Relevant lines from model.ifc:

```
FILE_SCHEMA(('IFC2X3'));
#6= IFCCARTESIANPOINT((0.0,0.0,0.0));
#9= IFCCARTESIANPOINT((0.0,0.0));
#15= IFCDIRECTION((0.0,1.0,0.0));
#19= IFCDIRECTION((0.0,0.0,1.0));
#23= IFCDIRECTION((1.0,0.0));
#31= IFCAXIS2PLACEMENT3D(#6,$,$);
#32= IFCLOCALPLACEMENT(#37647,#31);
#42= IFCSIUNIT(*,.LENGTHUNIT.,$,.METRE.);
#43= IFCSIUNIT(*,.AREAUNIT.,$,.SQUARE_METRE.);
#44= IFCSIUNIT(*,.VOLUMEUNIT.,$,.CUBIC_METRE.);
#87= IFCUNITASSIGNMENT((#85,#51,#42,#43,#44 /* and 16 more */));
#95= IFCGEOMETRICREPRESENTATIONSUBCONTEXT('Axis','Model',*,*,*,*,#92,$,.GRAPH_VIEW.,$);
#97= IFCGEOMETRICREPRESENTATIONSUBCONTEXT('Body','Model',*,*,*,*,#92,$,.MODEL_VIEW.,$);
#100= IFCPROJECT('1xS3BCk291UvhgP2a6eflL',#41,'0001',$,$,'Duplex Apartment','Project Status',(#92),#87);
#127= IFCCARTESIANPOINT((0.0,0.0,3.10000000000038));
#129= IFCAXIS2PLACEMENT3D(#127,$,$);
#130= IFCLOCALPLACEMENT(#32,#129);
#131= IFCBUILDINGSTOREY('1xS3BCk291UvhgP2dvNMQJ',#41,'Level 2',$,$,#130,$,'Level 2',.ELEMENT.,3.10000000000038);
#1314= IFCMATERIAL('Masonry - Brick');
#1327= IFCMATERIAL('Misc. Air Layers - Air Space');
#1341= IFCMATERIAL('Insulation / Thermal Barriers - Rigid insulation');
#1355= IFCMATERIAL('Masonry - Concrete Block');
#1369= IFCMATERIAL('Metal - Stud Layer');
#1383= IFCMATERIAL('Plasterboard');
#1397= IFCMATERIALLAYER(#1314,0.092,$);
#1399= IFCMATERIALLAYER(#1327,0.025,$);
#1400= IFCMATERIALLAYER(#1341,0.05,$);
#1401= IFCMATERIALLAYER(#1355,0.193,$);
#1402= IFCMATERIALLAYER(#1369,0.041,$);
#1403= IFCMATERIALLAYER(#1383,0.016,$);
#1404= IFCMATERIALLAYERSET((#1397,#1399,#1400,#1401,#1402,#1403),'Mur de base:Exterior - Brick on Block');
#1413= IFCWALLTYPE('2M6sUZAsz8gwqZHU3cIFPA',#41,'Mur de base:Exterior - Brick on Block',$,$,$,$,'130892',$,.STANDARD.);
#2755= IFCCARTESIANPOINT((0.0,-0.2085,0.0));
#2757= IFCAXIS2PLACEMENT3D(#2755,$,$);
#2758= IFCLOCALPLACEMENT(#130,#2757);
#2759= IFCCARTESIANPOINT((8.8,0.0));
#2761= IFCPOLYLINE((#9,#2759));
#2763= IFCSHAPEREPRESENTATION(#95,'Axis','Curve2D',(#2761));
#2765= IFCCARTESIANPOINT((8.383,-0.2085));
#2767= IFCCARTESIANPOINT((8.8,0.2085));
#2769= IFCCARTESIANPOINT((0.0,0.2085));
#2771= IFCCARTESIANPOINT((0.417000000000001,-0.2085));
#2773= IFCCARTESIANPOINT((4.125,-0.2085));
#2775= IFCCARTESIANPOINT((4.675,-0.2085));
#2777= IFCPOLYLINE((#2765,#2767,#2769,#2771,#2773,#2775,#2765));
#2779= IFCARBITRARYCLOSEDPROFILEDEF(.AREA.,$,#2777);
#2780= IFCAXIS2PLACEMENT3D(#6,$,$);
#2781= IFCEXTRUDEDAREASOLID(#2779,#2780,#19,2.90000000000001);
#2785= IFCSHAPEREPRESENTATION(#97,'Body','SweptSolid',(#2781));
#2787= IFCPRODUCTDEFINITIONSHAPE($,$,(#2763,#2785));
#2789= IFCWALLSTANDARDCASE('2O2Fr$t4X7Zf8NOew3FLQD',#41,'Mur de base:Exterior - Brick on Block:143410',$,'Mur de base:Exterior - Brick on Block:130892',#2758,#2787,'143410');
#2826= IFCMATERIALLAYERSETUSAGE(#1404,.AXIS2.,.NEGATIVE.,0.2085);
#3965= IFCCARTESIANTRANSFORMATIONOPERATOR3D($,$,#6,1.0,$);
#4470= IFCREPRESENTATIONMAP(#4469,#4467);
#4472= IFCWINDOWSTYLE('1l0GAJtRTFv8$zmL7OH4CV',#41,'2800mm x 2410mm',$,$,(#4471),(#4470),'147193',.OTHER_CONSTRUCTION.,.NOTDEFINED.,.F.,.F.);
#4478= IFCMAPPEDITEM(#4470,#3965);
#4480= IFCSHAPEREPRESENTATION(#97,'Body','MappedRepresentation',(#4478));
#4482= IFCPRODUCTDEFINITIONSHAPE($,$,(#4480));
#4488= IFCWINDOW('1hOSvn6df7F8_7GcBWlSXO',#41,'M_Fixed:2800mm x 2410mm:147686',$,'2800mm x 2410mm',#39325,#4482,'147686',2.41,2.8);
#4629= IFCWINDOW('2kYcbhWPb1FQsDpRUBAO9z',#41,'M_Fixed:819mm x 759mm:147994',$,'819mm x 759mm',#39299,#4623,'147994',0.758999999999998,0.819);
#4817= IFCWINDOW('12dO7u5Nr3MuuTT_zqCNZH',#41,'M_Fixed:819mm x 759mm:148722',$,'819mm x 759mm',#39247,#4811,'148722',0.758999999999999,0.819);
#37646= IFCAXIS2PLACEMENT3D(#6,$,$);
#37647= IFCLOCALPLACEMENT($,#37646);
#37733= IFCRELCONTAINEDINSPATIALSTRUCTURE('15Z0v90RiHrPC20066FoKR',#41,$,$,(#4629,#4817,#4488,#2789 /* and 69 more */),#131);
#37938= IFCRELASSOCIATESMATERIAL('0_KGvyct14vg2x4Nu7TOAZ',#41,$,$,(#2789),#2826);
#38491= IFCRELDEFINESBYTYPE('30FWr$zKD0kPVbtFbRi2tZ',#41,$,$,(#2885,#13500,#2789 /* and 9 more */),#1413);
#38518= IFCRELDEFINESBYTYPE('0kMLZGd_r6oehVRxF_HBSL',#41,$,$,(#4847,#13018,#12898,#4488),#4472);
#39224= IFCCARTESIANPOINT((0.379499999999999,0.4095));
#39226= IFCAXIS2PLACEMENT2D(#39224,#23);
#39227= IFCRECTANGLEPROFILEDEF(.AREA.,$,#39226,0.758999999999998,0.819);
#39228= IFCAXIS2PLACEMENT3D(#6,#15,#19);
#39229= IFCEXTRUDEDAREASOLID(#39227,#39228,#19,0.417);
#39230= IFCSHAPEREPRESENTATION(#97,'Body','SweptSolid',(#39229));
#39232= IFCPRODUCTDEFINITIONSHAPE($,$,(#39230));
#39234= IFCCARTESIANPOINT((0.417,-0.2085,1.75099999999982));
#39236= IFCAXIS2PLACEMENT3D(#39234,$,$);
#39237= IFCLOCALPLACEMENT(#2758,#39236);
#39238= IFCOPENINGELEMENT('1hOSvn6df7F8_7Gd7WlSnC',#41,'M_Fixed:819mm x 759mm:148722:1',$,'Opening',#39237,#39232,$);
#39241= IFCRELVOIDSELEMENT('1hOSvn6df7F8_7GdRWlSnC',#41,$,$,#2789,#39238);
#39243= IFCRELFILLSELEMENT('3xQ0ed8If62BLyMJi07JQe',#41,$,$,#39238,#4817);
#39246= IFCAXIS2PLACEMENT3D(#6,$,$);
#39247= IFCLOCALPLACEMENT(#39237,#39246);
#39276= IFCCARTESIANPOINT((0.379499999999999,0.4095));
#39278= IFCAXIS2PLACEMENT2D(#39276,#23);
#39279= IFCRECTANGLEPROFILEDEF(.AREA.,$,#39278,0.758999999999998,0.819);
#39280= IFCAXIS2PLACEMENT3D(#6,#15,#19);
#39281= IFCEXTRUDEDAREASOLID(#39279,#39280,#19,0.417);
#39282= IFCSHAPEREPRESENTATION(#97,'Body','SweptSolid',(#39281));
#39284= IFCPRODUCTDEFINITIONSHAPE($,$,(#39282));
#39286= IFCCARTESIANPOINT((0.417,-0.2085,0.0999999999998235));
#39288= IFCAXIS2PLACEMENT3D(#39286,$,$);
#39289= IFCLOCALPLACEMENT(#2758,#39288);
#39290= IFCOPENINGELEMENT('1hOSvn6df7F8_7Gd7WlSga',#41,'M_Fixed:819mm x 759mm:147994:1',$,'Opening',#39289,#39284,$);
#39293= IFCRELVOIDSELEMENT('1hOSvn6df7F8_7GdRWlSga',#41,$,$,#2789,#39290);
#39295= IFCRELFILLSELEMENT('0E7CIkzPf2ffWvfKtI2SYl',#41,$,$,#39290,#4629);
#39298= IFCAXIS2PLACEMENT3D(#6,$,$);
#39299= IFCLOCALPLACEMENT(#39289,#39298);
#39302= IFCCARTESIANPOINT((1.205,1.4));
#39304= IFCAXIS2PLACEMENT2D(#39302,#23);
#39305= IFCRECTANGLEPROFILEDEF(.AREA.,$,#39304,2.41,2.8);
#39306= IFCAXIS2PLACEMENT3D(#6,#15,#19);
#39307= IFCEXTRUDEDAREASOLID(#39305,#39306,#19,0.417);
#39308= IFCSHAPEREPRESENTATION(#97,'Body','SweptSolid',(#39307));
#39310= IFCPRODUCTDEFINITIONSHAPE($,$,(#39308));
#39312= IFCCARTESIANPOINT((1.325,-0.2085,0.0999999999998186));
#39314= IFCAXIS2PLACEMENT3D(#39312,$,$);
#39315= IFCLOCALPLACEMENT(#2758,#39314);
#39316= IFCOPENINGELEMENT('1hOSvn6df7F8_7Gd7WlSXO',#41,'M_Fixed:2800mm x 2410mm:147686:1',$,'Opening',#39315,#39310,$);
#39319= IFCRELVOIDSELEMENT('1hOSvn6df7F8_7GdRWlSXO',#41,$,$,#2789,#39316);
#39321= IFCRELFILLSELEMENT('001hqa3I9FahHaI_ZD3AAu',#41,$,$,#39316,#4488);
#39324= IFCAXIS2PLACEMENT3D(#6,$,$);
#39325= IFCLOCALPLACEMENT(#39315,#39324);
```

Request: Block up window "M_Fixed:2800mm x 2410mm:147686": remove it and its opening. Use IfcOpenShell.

```python
import ifcopenshell
import ifcopenshell.api.feature
import ifcopenshell.api.root
import ifcopenshell.geom
import ifcopenshell.util.shape

model = ifcopenshell.open("model.ifc")
settings = ifcopenshell.geom.settings()


def volume(element):
    """Net volume in cubic metres, openings subtracted."""
    shape = ifcopenshell.geom.create_shape(settings, element)
    return ifcopenshell.util.shape.get_volume(shape.geometry)


window = model.by_guid("1hOSvn6df7F8_7GcBWlSXO")
opening = window.FillsVoids[0].RelatingOpeningElement
wall = opening.VoidsElements[0].RelatingBuildingElement
before = volume(wall)

ifcopenshell.api.root.remove_product(model, product=window)
ifcopenshell.api.feature.remove_feature(model, feature=opening)

after = volume(wall)

print(f"wall volume {before:.3f} -> {after:.3f} m3")

model.write("model_v2.ifc")
```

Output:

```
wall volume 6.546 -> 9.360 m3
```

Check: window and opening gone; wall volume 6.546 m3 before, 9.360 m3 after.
